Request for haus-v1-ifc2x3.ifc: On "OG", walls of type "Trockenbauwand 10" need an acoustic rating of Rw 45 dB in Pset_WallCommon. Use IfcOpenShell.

First a look at what the model holds.

```python
import ifcopenshell
import ifcopenshell.util.element

model = ifcopenshell.open("haus-v1-ifc2x3.ifc")
print(model.schema)
storey = next(s for s in model.by_type("IfcBuildingStorey") if s.Name == "OG")
walls = [e for e in ifcopenshell.util.element.get_decomposition(storey) if e.is_a("IfcWall")]
seen = {}
for e in walls:
    element_type = ifcopenshell.util.element.get_type(e)
    key = (element_type.Name if element_type != e and element_type else None, ifcopenshell.util.element.get_pset(e, "Pset_WallCommon", "AcousticRating"))
    seen[key] = seen.get(key, 0) + 1
for (name, value), count in sorted(seen.items(), key=str):
    print(count, "x", name, "|", value)
```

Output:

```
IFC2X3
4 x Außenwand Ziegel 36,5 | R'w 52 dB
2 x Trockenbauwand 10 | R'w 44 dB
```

```python
import ifcopenshell
import ifcopenshell.api.pset
import ifcopenshell.util.element

model = ifcopenshell.open("haus-v1-ifc2x3.ifc")

storey = next(s for s in model.by_type("IfcBuildingStorey") if s.Name == "OG")
walls = [e for e in ifcopenshell.util.element.get_decomposition(storey) if e.is_a("IfcWall")]

count = 0
for e in walls:
    element_type = ifcopenshell.util.element.get_type(e)
    if element_type in (None, e) or element_type.Name != "Trockenbauwand 10":
        continue
    # add_pset returns the element's existing set when there is one.
    pset = ifcopenshell.api.pset.add_pset(model, product=e, name="Pset_WallCommon")
    ifcopenshell.api.pset.edit_pset(model, pset=pset, properties={"AcousticRating": "Rw 45 dB"})
    count += 1

print(count, "walls updated")

model.write("haus-v1-ifc2x3_v2.ifc")
```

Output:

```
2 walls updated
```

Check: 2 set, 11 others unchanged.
